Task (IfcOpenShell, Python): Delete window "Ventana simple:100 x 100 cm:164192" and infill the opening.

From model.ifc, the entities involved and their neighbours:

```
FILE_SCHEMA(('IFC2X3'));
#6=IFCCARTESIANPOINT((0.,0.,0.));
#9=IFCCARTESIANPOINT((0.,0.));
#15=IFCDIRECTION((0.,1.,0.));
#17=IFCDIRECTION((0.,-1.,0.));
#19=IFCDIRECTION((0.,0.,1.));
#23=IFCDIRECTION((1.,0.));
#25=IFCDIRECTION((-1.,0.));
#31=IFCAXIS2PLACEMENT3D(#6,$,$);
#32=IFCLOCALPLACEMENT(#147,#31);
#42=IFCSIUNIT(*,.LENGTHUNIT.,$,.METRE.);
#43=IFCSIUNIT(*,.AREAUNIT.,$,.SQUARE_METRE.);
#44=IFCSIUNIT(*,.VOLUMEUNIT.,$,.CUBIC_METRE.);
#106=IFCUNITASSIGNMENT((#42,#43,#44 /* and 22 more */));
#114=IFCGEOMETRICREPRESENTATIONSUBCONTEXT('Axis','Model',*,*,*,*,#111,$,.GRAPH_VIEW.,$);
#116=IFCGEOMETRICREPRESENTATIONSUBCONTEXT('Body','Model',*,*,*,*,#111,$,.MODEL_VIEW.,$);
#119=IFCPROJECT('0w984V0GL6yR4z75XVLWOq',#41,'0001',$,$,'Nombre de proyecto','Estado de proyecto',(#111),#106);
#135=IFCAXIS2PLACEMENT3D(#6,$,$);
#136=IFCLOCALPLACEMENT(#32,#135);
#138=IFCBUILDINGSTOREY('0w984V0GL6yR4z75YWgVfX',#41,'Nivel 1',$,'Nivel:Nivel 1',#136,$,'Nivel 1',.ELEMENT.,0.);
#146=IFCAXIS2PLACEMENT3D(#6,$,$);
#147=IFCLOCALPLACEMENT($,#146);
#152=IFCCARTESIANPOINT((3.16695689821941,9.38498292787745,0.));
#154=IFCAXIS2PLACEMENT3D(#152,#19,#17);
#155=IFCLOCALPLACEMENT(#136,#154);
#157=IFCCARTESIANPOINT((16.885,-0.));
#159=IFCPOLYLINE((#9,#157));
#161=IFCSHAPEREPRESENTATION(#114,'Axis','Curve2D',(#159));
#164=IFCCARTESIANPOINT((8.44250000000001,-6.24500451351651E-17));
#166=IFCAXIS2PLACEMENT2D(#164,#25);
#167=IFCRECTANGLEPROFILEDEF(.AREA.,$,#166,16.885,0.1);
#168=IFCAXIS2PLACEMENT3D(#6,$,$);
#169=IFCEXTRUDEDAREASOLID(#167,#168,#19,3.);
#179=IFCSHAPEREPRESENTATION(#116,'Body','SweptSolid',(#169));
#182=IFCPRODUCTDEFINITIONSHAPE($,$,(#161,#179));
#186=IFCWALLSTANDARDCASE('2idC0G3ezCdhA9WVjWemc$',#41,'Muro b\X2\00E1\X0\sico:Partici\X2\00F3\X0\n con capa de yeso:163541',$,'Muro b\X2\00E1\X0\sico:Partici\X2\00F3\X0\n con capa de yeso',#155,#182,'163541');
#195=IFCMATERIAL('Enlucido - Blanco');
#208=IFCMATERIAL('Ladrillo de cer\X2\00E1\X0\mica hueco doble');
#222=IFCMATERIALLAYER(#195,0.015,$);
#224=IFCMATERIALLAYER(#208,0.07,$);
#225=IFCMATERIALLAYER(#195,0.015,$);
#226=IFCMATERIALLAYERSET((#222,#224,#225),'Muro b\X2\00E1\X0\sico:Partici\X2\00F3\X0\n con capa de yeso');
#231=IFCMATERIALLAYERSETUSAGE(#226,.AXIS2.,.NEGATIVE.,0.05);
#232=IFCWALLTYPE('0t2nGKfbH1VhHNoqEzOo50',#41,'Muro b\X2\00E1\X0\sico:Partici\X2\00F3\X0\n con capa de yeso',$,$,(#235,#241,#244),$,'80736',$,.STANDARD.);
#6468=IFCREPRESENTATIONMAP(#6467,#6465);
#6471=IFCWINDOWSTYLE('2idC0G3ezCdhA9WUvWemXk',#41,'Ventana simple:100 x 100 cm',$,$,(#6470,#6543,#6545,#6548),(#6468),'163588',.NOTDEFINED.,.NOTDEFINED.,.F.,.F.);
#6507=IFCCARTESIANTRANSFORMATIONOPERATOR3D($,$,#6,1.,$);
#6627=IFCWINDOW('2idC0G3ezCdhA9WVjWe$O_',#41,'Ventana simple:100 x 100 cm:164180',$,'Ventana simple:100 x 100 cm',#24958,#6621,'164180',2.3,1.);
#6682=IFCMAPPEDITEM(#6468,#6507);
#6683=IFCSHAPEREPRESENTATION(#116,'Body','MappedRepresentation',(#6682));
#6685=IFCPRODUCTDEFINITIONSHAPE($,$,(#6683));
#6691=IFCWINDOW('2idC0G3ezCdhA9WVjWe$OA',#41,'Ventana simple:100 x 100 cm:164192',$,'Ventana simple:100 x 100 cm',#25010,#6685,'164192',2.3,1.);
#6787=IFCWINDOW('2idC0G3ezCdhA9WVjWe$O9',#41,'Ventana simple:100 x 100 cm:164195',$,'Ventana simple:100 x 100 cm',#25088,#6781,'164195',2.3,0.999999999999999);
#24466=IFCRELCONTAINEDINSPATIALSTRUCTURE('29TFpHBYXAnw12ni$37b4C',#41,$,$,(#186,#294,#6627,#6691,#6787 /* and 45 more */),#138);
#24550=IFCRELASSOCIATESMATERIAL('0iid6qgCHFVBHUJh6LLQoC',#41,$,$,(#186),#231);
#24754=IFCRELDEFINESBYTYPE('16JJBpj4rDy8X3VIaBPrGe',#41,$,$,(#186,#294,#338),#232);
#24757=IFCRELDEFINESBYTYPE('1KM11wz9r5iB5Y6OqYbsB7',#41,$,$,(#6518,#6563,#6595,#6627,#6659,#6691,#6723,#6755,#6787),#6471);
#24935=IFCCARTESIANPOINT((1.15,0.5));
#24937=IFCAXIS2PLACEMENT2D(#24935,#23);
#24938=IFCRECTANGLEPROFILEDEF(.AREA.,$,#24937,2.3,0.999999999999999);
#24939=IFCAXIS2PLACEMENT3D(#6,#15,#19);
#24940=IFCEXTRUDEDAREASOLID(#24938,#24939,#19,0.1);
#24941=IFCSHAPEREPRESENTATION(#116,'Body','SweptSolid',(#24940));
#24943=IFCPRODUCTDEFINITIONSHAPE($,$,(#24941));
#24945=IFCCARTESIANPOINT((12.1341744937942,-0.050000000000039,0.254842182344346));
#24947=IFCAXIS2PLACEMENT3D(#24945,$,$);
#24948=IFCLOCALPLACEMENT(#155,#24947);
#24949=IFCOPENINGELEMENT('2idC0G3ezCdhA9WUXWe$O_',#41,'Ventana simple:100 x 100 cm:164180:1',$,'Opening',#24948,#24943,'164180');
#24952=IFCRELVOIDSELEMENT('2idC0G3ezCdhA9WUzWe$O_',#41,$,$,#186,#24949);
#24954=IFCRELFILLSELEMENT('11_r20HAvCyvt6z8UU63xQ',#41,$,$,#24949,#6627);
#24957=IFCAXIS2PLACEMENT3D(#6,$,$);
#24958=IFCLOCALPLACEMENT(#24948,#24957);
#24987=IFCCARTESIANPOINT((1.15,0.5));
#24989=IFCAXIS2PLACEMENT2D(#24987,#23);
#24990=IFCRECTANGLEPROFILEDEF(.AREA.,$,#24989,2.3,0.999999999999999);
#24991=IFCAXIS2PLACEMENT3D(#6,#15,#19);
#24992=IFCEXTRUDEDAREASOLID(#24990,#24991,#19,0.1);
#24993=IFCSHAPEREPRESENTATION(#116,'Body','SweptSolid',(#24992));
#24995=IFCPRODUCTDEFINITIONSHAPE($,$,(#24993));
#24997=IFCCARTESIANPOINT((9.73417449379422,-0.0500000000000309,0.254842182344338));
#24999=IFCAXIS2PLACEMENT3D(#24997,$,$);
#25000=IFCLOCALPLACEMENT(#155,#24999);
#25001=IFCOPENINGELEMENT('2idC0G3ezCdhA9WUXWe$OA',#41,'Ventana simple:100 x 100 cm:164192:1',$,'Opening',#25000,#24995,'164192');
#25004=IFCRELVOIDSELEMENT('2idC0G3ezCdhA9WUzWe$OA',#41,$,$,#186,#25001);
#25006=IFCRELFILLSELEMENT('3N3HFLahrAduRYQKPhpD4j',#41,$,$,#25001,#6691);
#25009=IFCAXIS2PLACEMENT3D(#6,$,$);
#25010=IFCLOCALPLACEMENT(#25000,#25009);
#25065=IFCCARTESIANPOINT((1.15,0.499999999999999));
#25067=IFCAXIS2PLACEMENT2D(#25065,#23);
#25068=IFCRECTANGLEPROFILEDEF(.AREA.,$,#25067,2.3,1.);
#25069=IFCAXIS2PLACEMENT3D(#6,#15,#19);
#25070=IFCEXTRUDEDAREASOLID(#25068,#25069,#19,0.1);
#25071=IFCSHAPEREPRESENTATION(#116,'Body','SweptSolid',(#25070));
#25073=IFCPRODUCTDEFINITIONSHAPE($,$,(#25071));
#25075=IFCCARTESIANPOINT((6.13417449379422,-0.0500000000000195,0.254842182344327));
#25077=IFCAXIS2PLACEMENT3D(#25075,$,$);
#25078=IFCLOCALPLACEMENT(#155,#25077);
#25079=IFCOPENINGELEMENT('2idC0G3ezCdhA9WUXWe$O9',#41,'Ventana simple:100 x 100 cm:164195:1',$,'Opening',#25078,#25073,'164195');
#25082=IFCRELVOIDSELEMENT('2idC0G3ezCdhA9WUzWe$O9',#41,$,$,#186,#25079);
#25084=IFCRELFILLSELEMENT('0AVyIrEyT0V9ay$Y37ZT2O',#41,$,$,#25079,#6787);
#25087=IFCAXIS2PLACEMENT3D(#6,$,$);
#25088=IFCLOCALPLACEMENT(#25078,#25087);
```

```python
import ifcopenshell
import ifcopenshell.api.feature
import ifcopenshell.api.root
import ifcopenshell.geom
import ifcopenshell.util.shape

model = ifcopenshell.open("model.ifc")
settings = ifcopenshell.geom.settings()


def volume(element):
    """Net volume in cubic metres, openings subtracted."""
    shape = ifcopenshell.geom.create_shape(settings, element)
    return ifcopenshell.util.shape.get_volume(shape.geometry)


window = model.by_guid("2idC0G3ezCdhA9WVjWe$OA")
opening = window.FillsVoids[0].RelatingOpeningElement
wall = opening.VoidsElements[0].RelatingBuildingElement
before = volume(wall)

ifcopenshell.api.root.remove_product(model, product=window)
ifcopenshell.api.feature.remove_feature(model, feature=opening)

after = volume(wall)

print(f"wall volume {before:.3f} -> {after:.3f} m3")

model.write("model_updated.ifc")
```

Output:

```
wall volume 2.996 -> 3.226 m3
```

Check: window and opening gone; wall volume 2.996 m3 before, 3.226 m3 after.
